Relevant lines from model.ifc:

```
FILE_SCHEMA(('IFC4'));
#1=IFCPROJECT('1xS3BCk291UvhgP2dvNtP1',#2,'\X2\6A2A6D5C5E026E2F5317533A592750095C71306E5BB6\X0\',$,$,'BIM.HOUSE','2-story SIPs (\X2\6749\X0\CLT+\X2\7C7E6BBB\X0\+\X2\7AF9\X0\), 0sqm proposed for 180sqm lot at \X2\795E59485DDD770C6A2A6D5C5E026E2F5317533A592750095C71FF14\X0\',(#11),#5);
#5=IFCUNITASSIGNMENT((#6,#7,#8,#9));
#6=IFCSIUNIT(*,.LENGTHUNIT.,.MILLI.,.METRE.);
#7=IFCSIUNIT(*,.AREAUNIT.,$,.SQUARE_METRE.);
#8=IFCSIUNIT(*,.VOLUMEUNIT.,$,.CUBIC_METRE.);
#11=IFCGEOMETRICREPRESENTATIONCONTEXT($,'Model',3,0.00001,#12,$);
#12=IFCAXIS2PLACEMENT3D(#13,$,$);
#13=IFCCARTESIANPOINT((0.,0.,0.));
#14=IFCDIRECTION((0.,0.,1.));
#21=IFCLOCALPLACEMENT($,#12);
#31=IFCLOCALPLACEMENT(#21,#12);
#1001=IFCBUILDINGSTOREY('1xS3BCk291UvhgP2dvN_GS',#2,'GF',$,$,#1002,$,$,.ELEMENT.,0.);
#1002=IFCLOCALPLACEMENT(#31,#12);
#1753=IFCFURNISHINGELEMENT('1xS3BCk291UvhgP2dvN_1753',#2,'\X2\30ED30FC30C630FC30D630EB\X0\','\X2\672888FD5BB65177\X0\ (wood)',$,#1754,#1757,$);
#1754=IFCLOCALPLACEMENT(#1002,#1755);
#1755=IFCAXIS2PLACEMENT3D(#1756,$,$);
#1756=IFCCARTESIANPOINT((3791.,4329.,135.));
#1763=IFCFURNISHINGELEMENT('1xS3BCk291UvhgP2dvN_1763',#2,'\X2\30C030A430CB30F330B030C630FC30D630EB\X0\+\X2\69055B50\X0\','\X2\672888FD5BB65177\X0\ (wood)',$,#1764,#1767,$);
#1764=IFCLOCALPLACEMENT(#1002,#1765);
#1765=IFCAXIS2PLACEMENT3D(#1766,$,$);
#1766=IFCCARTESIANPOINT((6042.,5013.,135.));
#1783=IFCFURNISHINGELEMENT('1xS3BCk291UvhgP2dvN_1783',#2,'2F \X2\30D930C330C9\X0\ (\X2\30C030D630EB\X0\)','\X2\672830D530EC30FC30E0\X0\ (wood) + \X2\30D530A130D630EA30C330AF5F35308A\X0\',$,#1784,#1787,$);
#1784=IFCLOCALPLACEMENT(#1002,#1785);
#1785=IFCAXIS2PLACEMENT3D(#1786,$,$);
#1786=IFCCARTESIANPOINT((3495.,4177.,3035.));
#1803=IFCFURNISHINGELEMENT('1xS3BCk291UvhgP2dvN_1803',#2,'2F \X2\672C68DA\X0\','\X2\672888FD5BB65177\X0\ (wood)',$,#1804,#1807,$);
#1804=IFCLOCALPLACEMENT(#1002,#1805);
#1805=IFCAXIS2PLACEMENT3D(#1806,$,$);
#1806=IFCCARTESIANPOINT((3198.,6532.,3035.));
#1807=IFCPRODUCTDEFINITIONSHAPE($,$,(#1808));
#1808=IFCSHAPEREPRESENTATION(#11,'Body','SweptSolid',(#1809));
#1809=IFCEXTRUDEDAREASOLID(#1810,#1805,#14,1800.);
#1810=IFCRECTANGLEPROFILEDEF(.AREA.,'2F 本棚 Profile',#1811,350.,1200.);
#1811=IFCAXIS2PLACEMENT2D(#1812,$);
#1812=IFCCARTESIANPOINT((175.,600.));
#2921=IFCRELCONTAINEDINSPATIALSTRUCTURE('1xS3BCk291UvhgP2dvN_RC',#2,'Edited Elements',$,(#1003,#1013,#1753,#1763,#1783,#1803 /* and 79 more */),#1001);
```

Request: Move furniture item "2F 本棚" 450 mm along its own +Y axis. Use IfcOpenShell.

```python
import ifcopenshell
import ifcopenshell.api.geometry
import ifcopenshell.util.placement

model = ifcopenshell.open("model.ifc")

item = model.by_guid("1xS3BCk291UvhgP2dvN_1803")
matrix = ifcopenshell.util.placement.get_local_placement(item.ObjectPlacement)
matrix[:3, 3] += matrix[:3, 1] * 450.0
ifcopenshell.api.geometry.edit_object_placement(model, product=item, matrix=matrix, is_si=False)

print(ifcopenshell.util.placement.get_local_placement(item.ObjectPlacement).round(3) + 0.0)

model.write("model_updated.ifc")
```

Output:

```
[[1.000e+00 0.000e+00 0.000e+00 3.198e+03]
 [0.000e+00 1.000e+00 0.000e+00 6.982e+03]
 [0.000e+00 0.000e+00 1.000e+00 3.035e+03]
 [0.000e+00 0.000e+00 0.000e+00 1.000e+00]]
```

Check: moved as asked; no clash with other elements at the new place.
